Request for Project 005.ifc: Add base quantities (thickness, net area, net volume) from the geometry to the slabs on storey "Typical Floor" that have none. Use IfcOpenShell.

First a look at what the model holds.

```python
import ifcopenshell
import ifcopenshell.util.element
import ifcopenshell.util.unit

model = ifcopenshell.open("Project 005.ifc")
print(model.schema)
for unit_type in ("LENGTHUNIT", "AREAUNIT", "VOLUMEUNIT"):
    print(unit_type, ifcopenshell.util.unit.calculate_unit_scale(model, unit_type))
storey = next(s for s in model.by_type("IfcBuildingStorey") if s.Name == "Typical Floor")
slabs = [e for e in ifcopenshell.util.element.get_decomposition(storey) if e.is_a("IfcSlab")]
for e in sorted(slabs, key=lambda e: e.id()):
    print(e.id(), e.is_a(), e.Name, list(ifcopenshell.util.element.get_psets(e, qtos_only=True)), sep=" | ")
```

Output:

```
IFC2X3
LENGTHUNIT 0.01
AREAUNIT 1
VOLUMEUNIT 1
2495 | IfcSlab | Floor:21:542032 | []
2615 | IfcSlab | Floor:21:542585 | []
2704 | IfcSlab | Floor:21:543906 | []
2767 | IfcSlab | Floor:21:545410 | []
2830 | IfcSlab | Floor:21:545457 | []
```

```python
import ifcopenshell
import ifcopenshell.api.pset
import ifcopenshell.geom
import ifcopenshell.util.element
import ifcopenshell.util.shape
import ifcopenshell.util.unit

model = ifcopenshell.open("Project 005.ifc")
unit_scale = ifcopenshell.util.unit.calculate_unit_scale(model)
area_scale = ifcopenshell.util.unit.calculate_unit_scale(model, "AREAUNIT")
volume_scale = ifcopenshell.util.unit.calculate_unit_scale(model, "VOLUMEUNIT")
settings = ifcopenshell.geom.settings()

storey = next(s for s in model.by_type("IfcBuildingStorey") if s.Name == "Typical Floor")
slabs = [e for e in ifcopenshell.util.element.get_decomposition(storey) if e.is_a("IfcSlab")]

for e in sorted(slabs, key=lambda e: e.id()):
    if ifcopenshell.util.element.get_psets(e, qtos_only=True, should_inherit=False):
        continue
    # Geometry comes back in metres, in the element's own axes.
    shape = ifcopenshell.geom.create_shape(settings, e)
    values = {
        "Width": ifcopenshell.util.shape.get_z(shape.geometry) / unit_scale,
        "NetArea": ifcopenshell.util.shape.get_footprint_area(shape.geometry) / area_scale,
        "NetVolume": ifcopenshell.util.shape.get_volume(shape.geometry) / volume_scale,
    }
    qto = ifcopenshell.api.pset.add_qto(model, product=e, name="BaseQuantities")
    ifcopenshell.api.pset.edit_qto(model, qto=qto, properties=values)
    print(e.id(), {k: round(v, 3) for k, v in values.items()})

model.write("Project 005_rev.ifc")
```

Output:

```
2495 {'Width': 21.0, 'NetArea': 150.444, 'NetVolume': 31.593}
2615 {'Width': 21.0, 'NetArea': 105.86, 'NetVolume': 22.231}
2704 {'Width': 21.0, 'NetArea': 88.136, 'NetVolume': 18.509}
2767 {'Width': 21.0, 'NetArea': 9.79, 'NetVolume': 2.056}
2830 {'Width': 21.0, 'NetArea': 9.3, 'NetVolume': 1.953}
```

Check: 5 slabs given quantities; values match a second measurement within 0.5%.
